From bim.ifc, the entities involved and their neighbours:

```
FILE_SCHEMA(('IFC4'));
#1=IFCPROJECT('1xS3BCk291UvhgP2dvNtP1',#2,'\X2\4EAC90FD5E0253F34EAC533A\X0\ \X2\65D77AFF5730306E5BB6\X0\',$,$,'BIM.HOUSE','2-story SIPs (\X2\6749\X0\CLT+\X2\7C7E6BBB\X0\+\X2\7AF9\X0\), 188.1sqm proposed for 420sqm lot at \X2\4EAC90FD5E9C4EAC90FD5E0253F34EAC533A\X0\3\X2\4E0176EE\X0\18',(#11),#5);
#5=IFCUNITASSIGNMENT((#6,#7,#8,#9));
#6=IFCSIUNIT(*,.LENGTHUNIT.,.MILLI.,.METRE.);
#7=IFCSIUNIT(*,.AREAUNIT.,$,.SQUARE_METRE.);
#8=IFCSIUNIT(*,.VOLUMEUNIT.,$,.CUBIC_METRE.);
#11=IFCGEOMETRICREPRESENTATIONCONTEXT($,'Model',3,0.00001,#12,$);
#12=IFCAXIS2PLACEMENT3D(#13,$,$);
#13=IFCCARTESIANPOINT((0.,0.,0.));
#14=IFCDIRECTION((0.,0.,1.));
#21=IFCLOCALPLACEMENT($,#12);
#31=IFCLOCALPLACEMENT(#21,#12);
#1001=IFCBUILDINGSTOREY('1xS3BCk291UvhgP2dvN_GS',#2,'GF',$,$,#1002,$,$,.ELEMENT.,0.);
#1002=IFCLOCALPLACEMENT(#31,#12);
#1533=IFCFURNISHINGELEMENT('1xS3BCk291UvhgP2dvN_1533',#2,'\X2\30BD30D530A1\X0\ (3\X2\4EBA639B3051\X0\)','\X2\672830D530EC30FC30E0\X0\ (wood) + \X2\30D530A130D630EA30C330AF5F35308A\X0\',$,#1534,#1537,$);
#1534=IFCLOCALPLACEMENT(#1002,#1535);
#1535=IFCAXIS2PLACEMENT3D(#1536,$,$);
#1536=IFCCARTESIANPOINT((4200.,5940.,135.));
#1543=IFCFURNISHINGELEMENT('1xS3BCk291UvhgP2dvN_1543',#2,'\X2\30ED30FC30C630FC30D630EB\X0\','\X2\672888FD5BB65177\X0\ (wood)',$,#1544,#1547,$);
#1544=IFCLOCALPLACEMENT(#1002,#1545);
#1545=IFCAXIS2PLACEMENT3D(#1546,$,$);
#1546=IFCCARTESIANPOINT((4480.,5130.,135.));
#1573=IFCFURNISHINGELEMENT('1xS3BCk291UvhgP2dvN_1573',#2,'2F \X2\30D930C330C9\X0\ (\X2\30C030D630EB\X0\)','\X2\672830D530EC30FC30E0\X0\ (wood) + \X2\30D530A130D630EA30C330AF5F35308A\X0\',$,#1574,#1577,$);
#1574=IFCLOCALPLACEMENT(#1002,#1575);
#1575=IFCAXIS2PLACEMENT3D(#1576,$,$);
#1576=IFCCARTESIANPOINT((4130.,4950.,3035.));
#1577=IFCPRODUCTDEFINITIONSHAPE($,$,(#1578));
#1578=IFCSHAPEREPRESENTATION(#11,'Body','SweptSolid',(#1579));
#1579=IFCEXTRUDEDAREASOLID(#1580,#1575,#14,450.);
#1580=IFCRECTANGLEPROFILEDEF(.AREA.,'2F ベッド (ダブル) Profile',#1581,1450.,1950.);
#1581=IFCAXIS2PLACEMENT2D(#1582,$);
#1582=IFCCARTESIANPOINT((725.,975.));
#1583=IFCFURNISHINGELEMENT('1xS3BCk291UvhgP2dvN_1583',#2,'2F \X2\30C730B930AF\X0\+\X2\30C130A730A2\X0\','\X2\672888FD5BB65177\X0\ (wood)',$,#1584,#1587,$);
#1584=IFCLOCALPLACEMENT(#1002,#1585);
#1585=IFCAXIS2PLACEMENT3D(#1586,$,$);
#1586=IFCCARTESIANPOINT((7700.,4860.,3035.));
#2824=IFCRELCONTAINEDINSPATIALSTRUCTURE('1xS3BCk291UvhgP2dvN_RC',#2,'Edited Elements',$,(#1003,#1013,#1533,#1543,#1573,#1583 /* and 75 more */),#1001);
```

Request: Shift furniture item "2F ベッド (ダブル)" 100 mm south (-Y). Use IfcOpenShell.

```python
import ifcopenshell
import ifcopenshell.api.geometry
import ifcopenshell.util.placement
import ifcopenshell.util.unit

model = ifcopenshell.open("bim.ifc")
unit_scale = ifcopenshell.util.unit.calculate_unit_scale(model)

item = model.by_guid("1xS3BCk291UvhgP2dvN_1573")
matrix = ifcopenshell.util.placement.get_local_placement(item.ObjectPlacement)
matrix[1, 3] -= 0.1 / unit_scale
ifcopenshell.api.geometry.edit_object_placement(model, product=item, matrix=matrix, is_si=False)

print(ifcopenshell.util.placement.get_local_placement(item.ObjectPlacement).round(3) + 0.0)

model.write("bim_edited.ifc")
```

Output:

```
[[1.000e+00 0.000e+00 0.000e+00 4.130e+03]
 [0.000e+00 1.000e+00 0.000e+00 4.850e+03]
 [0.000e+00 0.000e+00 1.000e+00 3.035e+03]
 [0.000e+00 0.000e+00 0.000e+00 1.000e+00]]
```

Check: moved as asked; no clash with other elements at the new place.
